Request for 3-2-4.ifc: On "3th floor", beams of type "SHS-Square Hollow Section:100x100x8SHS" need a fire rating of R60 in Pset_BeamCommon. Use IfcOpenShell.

First a look at what the model holds.

```python
import ifcopenshell
import ifcopenshell.util.element

model = ifcopenshell.open("3-2-4.ifc")
print(model.schema)
storey = next(s for s in model.by_type("IfcBuildingStorey") if s.Name == "3th floor")
beams = [e for e in ifcopenshell.util.element.get_decomposition(storey) if e.is_a("IfcBeam")]
seen = {}
for e in beams:
    element_type = ifcopenshell.util.element.get_type(e)
    key = (element_type.Name if element_type != e and element_type else None, ifcopenshell.util.element.get_pset(e, "Pset_BeamCommon", "FireRating"))
    seen[key] = seen.get(key, 0) + 1
for (name, value), count in sorted(seen.items(), key=str):
    print(count, "x", name, "|", value)
```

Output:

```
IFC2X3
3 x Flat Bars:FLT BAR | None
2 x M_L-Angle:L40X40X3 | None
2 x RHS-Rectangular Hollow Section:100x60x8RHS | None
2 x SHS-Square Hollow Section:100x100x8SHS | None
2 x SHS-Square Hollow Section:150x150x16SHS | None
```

```python
import ifcopenshell
import ifcopenshell.api.pset
import ifcopenshell.util.element

model = ifcopenshell.open("3-2-4.ifc")

storey = next(s for s in model.by_type("IfcBuildingStorey") if s.Name == "3th floor")
beams = [e for e in ifcopenshell.util.element.get_decomposition(storey) if e.is_a("IfcBeam")]

count = 0
for e in beams:
    element_type = ifcopenshell.util.element.get_type(e)
    if element_type in (None, e) or element_type.Name != "SHS-Square Hollow Section:100x100x8SHS":
        continue
    # add_pset returns the element's existing set when there is one.
    pset = ifcopenshell.api.pset.add_pset(model, product=e, name="Pset_BeamCommon")
    ifcopenshell.api.pset.edit_pset(model, pset=pset, properties={"FireRating": "R60"})
    count += 1

print(count, "beams updated")

model.write("3-2-4_edited.ifc")
```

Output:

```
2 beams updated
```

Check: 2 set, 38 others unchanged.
